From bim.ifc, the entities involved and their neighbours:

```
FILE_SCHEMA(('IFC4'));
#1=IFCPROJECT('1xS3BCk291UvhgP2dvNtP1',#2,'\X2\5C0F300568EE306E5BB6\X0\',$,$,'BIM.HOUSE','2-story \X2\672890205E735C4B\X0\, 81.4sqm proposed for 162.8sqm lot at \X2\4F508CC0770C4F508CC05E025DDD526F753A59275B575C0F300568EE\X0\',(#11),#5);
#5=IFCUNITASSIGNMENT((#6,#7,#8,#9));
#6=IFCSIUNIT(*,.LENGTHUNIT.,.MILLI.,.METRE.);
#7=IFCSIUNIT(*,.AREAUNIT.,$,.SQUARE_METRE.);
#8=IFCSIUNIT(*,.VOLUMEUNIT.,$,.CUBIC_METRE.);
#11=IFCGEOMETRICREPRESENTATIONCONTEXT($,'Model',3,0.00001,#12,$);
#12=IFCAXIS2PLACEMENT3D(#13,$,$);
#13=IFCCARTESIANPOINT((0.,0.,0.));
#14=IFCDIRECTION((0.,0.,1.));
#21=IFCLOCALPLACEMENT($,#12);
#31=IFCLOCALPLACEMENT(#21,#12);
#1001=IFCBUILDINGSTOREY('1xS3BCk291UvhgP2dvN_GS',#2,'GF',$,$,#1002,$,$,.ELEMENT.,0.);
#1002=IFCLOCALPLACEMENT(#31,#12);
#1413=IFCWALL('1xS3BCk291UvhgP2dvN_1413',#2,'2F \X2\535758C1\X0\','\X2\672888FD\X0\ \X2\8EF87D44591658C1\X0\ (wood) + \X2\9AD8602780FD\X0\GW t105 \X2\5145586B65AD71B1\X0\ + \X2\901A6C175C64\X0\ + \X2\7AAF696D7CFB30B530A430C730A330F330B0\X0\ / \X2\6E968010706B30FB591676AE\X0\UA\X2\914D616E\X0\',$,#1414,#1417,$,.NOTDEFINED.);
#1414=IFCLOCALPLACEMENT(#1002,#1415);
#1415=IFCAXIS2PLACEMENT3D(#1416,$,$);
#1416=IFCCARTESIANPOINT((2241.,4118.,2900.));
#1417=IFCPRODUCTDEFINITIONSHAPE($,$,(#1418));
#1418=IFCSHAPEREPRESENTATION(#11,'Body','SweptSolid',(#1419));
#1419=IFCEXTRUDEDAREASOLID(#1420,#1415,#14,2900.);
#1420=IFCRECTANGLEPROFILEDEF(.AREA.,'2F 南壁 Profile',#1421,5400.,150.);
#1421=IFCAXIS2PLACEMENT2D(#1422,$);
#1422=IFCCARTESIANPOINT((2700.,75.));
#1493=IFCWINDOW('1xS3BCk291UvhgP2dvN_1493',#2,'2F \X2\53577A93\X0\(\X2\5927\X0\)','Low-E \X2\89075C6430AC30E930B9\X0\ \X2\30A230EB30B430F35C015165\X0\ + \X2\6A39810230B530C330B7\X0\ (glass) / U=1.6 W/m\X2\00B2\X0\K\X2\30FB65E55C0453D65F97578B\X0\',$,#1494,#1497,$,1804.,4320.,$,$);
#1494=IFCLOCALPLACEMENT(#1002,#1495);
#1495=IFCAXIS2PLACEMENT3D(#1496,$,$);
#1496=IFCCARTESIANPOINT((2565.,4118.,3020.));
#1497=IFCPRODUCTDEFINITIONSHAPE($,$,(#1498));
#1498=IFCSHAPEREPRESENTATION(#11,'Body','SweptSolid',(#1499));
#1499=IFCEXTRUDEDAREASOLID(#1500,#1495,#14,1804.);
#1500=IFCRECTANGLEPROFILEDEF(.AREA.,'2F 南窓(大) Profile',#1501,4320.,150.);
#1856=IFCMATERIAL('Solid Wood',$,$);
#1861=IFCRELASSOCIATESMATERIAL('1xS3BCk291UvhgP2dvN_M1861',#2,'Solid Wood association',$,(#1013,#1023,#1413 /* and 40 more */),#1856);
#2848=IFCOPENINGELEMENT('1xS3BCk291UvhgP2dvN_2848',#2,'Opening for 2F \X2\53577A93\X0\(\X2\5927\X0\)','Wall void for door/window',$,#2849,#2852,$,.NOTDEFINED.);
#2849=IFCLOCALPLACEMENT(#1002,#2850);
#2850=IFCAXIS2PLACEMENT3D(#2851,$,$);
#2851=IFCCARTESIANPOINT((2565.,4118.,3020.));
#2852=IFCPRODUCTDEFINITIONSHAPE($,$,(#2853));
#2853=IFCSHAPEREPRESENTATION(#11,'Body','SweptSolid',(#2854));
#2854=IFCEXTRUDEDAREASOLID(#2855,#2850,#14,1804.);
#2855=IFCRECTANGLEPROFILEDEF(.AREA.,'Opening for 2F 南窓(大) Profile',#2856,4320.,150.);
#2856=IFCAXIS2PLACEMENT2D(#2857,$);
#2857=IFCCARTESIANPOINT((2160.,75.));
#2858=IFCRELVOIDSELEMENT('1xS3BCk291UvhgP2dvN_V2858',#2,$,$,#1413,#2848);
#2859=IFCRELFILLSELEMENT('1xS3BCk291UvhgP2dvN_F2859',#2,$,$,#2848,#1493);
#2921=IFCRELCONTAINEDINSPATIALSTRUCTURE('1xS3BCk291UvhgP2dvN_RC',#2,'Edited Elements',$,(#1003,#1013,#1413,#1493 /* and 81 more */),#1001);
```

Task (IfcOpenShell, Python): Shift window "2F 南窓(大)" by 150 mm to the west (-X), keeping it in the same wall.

```python
import ifcopenshell
import ifcopenshell.api.geometry
import ifcopenshell.util.placement

model = ifcopenshell.open("bim.ifc")

window = model.by_id(1493)
opening = window.FillsVoids[0].RelatingOpeningElement
wall = opening.VoidsElements[0].RelatingBuildingElement

wall_matrix = ifcopenshell.util.placement.get_local_placement(wall.ObjectPlacement)
shift = wall_matrix[:3, 0] * -150.0
before = ifcopenshell.util.placement.get_local_placement(window.ObjectPlacement)[:3, 3].copy()

# The window is not placed relative to its opening, so move both.
for product in (opening, window):
    matrix = ifcopenshell.util.placement.get_local_placement(product.ObjectPlacement)
    matrix[:3, 3] += shift
    ifcopenshell.api.geometry.edit_object_placement(model, product=product, matrix=matrix, is_si=False)

after = ifcopenshell.util.placement.get_local_placement(window.ObjectPlacement)[:3, 3]
print("window moved by", (after - before).round(3) + 0.0)

model.write("bim_edited.ifc")
```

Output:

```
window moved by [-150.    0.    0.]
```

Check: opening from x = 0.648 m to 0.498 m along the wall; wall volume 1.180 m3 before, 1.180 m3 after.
